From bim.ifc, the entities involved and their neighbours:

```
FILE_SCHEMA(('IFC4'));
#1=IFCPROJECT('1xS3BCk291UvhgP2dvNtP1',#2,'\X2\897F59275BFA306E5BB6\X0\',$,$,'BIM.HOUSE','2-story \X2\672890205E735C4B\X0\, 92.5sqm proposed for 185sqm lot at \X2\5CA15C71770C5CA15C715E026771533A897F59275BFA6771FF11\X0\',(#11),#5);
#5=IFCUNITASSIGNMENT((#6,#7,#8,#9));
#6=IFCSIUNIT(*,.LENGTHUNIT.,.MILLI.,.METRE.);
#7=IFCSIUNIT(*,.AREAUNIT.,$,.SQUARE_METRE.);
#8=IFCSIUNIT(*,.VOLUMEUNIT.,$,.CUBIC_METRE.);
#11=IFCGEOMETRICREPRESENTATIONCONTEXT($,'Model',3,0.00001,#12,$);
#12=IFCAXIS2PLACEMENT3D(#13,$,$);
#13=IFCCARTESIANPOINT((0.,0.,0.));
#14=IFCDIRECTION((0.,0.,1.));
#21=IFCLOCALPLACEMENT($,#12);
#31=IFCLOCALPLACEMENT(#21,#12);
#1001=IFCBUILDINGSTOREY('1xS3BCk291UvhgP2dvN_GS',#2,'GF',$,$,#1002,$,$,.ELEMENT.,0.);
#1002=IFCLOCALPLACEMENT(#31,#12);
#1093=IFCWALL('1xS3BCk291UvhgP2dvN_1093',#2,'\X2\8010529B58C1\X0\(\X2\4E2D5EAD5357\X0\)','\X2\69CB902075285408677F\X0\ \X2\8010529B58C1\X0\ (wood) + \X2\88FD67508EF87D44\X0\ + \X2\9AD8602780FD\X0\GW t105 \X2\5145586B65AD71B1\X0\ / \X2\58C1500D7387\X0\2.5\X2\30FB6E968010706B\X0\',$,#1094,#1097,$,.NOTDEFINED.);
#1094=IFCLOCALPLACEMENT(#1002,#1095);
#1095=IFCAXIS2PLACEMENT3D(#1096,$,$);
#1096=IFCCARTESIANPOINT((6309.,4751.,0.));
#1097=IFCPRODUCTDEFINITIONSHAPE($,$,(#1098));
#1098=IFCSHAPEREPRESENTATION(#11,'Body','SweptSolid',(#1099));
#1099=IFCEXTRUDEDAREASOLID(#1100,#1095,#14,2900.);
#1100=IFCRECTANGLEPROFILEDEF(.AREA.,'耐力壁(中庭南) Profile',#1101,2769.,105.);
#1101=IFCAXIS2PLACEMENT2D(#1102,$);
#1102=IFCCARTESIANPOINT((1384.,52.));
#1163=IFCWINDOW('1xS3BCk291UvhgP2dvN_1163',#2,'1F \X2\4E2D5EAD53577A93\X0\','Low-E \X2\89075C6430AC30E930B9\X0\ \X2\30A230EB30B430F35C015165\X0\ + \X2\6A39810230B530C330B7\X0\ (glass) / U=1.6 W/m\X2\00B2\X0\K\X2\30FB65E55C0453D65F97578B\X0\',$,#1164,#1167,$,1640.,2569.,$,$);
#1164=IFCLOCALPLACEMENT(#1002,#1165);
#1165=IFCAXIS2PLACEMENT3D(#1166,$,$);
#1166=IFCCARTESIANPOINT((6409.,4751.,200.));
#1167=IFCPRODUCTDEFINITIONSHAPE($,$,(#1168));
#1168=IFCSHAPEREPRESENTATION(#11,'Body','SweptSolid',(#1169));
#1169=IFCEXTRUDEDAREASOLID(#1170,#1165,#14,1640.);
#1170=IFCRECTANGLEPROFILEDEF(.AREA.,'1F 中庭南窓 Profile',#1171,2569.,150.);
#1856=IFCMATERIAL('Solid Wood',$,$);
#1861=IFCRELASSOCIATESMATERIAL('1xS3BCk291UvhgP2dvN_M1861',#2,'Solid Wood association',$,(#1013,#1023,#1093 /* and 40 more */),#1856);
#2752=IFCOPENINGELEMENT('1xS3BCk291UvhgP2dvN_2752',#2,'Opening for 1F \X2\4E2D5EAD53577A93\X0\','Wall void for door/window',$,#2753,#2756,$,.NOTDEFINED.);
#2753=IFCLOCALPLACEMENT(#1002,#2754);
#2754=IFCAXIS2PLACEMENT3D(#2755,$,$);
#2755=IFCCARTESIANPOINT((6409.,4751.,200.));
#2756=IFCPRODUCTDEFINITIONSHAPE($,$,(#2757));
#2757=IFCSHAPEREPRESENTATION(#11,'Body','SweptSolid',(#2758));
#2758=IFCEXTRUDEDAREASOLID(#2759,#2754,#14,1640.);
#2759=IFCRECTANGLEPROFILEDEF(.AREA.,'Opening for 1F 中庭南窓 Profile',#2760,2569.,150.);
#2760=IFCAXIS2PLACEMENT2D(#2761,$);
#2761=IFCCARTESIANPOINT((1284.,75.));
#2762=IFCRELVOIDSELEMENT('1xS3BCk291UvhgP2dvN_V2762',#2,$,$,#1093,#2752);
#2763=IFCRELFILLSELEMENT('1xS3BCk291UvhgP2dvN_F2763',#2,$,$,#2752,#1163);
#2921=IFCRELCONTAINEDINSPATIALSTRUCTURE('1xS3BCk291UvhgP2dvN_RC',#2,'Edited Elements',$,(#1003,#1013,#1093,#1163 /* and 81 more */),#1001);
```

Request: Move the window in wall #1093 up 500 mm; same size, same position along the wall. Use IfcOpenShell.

```python
import numpy as np
import ifcopenshell
import ifcopenshell.api.geometry
import ifcopenshell.util.placement
import ifcopenshell.util.unit

model = ifcopenshell.open("bim.ifc")
unit_scale = ifcopenshell.util.unit.calculate_unit_scale(model)

window = model.by_id(1163)
opening = window.FillsVoids[0].RelatingOpeningElement
dz = 500.0

shift = np.array([0.0, 0.0, dz])
# The window is not placed relative to its opening, so move both.
for product in (opening, window):
    matrix = ifcopenshell.util.placement.get_local_placement(product.ObjectPlacement)
    matrix[:3, 3] += shift
    ifcopenshell.api.geometry.edit_object_placement(model, product=product, matrix=matrix, is_si=False)

print(f"moved by {dz * unit_scale:+.3f} m")

model.write("bim_v2.ifc")
```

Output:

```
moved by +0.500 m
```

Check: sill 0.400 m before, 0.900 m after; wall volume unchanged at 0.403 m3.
